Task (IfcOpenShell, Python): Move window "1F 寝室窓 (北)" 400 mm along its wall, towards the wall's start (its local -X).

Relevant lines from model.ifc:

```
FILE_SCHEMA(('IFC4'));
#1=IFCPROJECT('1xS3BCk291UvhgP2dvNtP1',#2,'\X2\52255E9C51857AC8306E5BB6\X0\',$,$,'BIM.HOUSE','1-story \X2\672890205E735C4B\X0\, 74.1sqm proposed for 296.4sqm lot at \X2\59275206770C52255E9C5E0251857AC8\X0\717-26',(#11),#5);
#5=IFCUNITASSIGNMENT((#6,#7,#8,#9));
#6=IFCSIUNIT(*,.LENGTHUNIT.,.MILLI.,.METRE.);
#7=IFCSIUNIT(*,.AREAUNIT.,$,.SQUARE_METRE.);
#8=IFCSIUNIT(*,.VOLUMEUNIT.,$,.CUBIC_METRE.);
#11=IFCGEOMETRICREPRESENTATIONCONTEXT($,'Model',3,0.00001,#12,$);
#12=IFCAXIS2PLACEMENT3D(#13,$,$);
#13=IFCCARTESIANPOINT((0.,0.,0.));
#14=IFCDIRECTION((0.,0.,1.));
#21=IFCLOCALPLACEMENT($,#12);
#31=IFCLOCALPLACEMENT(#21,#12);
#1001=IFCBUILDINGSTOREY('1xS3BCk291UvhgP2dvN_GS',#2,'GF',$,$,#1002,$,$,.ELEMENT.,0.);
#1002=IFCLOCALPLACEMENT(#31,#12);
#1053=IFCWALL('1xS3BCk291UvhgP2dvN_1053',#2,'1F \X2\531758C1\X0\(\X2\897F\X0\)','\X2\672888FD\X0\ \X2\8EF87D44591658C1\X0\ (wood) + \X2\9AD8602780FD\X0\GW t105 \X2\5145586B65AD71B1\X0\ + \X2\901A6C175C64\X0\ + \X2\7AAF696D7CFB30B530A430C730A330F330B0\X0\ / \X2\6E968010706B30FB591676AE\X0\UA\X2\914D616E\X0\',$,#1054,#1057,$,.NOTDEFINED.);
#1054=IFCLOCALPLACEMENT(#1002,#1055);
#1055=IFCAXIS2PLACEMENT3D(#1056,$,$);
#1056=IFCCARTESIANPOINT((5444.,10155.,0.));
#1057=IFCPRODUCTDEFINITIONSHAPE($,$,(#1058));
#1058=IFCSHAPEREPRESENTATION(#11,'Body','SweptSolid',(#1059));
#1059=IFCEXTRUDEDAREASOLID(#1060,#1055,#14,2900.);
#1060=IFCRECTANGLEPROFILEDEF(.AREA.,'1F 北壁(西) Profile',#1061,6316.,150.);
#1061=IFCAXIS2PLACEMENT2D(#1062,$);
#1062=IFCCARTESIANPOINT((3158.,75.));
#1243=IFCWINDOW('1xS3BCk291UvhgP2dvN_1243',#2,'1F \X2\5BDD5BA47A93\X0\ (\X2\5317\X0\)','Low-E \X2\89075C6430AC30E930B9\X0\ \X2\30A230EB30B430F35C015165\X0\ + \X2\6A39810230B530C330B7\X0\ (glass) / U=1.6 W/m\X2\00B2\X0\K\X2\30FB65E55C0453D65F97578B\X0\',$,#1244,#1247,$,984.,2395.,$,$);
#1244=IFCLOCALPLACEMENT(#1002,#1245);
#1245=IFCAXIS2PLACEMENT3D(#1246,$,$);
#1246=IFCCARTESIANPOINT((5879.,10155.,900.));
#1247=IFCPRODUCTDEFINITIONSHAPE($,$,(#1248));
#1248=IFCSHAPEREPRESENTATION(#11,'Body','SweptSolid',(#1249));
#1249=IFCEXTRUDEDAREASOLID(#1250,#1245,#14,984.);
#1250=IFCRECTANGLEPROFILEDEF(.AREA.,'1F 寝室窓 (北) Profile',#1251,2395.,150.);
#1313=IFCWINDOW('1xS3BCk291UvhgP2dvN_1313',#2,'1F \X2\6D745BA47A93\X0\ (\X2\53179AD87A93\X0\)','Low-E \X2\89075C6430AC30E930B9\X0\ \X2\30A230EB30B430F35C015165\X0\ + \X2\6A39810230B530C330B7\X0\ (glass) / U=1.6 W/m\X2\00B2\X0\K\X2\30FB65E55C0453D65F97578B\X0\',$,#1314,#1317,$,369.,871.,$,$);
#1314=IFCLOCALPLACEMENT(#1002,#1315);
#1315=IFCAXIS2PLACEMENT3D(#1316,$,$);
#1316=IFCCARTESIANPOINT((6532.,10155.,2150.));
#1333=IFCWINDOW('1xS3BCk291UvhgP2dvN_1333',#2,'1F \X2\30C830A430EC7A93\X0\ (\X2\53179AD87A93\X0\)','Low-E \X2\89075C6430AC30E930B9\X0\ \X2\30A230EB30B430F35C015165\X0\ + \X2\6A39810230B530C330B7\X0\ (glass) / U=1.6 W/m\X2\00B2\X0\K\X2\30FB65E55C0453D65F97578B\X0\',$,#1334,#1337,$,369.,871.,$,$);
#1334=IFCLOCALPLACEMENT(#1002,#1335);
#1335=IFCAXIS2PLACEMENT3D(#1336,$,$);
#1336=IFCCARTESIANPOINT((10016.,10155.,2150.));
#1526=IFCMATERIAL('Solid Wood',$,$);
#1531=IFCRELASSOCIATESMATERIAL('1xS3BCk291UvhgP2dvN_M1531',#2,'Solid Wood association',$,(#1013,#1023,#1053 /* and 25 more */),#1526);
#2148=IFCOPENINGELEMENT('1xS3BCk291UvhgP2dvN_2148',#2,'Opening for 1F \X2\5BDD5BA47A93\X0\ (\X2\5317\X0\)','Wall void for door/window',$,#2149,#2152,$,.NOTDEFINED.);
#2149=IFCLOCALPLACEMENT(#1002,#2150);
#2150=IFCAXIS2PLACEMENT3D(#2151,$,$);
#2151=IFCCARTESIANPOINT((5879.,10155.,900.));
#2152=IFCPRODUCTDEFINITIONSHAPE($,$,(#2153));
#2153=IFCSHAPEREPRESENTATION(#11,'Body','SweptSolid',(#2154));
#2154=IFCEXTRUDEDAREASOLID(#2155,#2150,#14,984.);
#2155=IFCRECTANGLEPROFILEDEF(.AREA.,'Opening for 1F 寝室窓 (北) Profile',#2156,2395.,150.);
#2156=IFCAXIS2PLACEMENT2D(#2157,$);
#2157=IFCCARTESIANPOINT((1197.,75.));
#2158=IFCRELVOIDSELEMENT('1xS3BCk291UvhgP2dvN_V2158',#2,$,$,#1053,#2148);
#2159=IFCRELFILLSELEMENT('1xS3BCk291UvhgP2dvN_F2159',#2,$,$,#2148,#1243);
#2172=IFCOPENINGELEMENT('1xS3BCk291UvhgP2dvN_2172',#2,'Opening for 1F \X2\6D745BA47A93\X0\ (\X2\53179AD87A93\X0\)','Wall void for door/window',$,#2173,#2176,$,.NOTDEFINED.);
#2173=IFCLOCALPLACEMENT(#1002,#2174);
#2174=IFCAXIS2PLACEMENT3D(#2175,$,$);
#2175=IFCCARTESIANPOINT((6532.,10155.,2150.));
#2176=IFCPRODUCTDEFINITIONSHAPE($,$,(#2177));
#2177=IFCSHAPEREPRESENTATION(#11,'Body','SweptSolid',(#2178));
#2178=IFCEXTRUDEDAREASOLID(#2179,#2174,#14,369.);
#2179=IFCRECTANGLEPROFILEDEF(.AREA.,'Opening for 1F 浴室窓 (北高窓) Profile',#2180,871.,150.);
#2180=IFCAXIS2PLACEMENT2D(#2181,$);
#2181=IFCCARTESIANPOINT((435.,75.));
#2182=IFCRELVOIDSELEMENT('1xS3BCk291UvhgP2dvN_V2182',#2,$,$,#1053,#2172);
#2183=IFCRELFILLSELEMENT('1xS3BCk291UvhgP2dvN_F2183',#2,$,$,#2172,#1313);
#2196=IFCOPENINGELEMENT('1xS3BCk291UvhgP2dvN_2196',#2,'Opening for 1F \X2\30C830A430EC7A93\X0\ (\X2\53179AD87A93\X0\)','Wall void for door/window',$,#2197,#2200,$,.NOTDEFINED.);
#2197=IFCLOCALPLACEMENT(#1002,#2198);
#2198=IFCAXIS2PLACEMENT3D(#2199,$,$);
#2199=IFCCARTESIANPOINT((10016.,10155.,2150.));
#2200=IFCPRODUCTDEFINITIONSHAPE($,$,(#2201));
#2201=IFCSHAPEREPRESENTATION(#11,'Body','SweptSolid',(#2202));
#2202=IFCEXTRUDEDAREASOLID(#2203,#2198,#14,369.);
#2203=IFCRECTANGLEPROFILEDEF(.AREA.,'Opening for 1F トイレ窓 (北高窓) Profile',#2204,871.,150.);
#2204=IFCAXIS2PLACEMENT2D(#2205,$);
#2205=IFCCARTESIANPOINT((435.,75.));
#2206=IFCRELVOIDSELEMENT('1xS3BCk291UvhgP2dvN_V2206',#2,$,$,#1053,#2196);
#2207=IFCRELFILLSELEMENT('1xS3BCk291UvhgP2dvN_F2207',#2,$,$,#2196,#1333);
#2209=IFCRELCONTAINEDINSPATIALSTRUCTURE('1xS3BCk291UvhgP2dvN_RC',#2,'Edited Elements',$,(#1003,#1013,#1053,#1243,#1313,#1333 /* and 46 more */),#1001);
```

```python
import ifcopenshell
import ifcopenshell.api.geometry
import ifcopenshell.util.placement
import ifcopenshell.util.unit

model = ifcopenshell.open("model.ifc")
unit_scale = ifcopenshell.util.unit.calculate_unit_scale(model)

window = model.by_id(1243)
opening = window.FillsVoids[0].RelatingOpeningElement
wall = opening.VoidsElements[0].RelatingBuildingElement

wall_matrix = ifcopenshell.util.placement.get_local_placement(wall.ObjectPlacement)
shift = wall_matrix[:3, 0] * -0.4 / unit_scale
before = ifcopenshell.util.placement.get_local_placement(window.ObjectPlacement)[:3, 3].copy()

# The window is not placed relative to its opening, so move both.
for product in (opening, window):
    matrix = ifcopenshell.util.placement.get_local_placement(product.ObjectPlacement)
    matrix[:3, 3] += shift
    ifcopenshell.api.geometry.edit_object_placement(model, product=product, matrix=matrix, is_si=False)

after = ifcopenshell.util.placement.get_local_placement(window.ObjectPlacement)[:3, 3]
print("window moved by", (after - before).round(3) + 0.0)

model.write("model_v2.ifc")
```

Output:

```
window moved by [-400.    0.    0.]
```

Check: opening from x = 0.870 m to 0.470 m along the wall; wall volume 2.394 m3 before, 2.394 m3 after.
